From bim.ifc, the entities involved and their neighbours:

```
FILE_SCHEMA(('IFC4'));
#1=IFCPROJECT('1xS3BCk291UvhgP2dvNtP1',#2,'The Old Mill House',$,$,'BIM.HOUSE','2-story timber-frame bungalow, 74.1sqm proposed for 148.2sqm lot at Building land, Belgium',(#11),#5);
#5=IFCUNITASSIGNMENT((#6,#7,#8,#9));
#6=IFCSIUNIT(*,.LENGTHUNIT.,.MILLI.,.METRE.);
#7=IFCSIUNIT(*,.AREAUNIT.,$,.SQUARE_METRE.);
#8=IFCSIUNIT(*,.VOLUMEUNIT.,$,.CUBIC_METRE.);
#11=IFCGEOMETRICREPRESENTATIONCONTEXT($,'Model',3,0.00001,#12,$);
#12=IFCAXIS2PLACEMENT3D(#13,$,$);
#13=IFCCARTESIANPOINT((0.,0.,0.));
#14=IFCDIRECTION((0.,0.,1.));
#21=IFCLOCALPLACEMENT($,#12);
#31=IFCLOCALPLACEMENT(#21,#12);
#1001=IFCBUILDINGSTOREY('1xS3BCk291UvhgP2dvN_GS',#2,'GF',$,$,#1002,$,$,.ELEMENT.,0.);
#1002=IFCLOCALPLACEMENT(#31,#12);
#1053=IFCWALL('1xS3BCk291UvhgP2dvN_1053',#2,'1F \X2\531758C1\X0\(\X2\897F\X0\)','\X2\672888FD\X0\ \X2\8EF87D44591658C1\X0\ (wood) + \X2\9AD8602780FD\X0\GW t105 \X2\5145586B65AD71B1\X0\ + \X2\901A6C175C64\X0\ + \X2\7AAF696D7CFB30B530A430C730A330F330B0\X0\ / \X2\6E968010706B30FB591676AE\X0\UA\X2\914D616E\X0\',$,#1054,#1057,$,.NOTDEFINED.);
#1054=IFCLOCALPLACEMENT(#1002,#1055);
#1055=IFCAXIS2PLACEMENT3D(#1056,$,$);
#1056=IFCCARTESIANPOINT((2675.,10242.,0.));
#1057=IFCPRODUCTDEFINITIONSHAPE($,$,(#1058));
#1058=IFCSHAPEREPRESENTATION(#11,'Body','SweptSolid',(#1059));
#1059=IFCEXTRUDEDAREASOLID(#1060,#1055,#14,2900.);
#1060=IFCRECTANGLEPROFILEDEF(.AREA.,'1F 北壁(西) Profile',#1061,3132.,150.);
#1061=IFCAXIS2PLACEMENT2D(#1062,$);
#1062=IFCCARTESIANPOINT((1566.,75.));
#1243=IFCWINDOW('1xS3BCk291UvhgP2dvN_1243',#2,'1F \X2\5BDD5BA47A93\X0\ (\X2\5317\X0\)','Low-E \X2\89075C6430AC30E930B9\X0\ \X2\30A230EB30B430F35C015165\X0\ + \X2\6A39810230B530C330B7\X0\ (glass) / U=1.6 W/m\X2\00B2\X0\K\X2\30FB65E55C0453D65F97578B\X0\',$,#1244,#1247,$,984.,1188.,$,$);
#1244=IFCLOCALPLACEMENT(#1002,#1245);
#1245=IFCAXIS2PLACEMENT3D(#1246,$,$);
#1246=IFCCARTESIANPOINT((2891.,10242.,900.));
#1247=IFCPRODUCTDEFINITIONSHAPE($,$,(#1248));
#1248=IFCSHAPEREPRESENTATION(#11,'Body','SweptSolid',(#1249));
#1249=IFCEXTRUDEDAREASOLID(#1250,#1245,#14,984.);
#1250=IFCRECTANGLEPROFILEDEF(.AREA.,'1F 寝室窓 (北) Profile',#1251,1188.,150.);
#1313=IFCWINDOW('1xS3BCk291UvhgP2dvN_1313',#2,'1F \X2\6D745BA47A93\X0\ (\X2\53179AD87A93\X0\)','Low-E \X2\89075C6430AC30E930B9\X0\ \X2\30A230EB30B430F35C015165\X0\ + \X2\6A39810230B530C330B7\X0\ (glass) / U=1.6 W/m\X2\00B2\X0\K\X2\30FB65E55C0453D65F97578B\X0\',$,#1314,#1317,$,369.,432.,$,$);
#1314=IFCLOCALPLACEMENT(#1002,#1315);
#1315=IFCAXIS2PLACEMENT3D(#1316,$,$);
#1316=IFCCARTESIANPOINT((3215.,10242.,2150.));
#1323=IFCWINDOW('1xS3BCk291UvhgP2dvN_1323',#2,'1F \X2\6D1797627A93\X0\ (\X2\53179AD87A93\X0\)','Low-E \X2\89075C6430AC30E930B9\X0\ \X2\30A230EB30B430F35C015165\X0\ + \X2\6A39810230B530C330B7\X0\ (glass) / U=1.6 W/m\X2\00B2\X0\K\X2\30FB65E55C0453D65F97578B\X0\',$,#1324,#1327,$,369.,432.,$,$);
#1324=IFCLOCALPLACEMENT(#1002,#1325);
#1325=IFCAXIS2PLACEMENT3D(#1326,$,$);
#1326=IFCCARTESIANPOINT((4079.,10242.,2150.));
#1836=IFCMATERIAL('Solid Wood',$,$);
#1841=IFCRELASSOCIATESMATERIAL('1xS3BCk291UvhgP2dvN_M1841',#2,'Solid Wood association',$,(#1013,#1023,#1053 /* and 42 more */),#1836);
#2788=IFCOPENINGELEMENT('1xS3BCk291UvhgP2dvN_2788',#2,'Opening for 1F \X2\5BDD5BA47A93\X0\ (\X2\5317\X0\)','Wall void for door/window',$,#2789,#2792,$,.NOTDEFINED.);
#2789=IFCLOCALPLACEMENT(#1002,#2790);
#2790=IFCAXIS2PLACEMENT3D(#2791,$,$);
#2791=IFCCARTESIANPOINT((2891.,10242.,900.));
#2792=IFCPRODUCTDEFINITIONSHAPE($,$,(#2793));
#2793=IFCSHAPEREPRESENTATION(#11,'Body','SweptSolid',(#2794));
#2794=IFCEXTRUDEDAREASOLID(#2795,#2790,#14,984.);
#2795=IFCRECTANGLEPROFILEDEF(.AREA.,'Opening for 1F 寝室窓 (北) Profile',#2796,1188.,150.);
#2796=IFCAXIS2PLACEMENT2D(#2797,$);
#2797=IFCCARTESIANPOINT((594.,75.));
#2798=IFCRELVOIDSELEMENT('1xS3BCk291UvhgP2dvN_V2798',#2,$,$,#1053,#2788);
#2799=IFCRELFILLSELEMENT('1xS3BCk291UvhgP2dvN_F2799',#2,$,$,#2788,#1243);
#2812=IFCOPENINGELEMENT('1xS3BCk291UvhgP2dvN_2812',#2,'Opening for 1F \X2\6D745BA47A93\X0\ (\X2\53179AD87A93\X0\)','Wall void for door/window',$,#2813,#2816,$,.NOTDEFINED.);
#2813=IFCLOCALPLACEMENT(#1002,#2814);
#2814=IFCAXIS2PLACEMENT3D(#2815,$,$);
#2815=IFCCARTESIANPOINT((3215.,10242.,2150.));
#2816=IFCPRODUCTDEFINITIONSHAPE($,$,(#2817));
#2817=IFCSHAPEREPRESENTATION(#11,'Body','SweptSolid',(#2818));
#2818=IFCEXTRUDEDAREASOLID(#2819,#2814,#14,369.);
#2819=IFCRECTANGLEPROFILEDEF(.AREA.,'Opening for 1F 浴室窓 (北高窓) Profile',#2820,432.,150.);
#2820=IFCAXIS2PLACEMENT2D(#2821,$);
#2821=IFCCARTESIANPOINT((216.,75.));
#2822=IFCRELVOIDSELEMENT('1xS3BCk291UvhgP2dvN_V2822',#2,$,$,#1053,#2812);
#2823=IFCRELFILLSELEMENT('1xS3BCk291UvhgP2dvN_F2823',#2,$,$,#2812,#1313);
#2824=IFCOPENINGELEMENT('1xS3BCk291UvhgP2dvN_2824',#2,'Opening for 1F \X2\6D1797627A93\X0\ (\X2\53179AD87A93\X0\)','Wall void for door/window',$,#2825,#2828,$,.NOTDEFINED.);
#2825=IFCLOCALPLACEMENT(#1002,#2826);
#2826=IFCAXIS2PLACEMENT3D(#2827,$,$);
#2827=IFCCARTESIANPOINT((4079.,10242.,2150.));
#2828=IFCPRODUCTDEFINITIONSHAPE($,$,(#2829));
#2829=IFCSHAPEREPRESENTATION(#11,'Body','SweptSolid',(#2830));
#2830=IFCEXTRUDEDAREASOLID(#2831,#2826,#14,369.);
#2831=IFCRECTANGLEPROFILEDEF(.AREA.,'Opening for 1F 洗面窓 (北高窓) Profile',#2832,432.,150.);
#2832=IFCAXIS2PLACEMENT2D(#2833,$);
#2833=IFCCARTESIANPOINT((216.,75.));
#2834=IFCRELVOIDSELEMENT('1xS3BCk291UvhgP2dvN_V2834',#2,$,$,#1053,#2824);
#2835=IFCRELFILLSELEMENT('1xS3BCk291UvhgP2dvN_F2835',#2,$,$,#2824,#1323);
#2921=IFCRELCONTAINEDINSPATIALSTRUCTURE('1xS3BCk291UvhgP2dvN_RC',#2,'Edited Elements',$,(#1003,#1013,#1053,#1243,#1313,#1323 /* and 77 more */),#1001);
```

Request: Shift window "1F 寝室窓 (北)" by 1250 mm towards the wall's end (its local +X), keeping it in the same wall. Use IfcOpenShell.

```python
import ifcopenshell
import ifcopenshell.api.geometry
import ifcopenshell.util.placement
import ifcopenshell.util.unit

model = ifcopenshell.open("bim.ifc")
unit_scale = ifcopenshell.util.unit.calculate_unit_scale(model)

window = model.by_id(1243)
opening = window.FillsVoids[0].RelatingOpeningElement
wall = opening.VoidsElements[0].RelatingBuildingElement

wall_matrix = ifcopenshell.util.placement.get_local_placement(wall.ObjectPlacement)
shift = wall_matrix[:3, 0] * 1.25 / unit_scale
before = ifcopenshell.util.placement.get_local_placement(window.ObjectPlacement)[:3, 3].copy()

# The window is not placed relative to its opening, so move both.
for product in (opening, window):
    matrix = ifcopenshell.util.placement.get_local_placement(product.ObjectPlacement)
    matrix[:3, 3] += shift
    ifcopenshell.api.geometry.edit_object_placement(model, product=product, matrix=matrix, is_si=False)

after = ifcopenshell.util.placement.get_local_placement(window.ObjectPlacement)[:3, 3]
print("window moved by", (after - before).round(3) + 0.0)

model.write("bim_rev.ifc")
```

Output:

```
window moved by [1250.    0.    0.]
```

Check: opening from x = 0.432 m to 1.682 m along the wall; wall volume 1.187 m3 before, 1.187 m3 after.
